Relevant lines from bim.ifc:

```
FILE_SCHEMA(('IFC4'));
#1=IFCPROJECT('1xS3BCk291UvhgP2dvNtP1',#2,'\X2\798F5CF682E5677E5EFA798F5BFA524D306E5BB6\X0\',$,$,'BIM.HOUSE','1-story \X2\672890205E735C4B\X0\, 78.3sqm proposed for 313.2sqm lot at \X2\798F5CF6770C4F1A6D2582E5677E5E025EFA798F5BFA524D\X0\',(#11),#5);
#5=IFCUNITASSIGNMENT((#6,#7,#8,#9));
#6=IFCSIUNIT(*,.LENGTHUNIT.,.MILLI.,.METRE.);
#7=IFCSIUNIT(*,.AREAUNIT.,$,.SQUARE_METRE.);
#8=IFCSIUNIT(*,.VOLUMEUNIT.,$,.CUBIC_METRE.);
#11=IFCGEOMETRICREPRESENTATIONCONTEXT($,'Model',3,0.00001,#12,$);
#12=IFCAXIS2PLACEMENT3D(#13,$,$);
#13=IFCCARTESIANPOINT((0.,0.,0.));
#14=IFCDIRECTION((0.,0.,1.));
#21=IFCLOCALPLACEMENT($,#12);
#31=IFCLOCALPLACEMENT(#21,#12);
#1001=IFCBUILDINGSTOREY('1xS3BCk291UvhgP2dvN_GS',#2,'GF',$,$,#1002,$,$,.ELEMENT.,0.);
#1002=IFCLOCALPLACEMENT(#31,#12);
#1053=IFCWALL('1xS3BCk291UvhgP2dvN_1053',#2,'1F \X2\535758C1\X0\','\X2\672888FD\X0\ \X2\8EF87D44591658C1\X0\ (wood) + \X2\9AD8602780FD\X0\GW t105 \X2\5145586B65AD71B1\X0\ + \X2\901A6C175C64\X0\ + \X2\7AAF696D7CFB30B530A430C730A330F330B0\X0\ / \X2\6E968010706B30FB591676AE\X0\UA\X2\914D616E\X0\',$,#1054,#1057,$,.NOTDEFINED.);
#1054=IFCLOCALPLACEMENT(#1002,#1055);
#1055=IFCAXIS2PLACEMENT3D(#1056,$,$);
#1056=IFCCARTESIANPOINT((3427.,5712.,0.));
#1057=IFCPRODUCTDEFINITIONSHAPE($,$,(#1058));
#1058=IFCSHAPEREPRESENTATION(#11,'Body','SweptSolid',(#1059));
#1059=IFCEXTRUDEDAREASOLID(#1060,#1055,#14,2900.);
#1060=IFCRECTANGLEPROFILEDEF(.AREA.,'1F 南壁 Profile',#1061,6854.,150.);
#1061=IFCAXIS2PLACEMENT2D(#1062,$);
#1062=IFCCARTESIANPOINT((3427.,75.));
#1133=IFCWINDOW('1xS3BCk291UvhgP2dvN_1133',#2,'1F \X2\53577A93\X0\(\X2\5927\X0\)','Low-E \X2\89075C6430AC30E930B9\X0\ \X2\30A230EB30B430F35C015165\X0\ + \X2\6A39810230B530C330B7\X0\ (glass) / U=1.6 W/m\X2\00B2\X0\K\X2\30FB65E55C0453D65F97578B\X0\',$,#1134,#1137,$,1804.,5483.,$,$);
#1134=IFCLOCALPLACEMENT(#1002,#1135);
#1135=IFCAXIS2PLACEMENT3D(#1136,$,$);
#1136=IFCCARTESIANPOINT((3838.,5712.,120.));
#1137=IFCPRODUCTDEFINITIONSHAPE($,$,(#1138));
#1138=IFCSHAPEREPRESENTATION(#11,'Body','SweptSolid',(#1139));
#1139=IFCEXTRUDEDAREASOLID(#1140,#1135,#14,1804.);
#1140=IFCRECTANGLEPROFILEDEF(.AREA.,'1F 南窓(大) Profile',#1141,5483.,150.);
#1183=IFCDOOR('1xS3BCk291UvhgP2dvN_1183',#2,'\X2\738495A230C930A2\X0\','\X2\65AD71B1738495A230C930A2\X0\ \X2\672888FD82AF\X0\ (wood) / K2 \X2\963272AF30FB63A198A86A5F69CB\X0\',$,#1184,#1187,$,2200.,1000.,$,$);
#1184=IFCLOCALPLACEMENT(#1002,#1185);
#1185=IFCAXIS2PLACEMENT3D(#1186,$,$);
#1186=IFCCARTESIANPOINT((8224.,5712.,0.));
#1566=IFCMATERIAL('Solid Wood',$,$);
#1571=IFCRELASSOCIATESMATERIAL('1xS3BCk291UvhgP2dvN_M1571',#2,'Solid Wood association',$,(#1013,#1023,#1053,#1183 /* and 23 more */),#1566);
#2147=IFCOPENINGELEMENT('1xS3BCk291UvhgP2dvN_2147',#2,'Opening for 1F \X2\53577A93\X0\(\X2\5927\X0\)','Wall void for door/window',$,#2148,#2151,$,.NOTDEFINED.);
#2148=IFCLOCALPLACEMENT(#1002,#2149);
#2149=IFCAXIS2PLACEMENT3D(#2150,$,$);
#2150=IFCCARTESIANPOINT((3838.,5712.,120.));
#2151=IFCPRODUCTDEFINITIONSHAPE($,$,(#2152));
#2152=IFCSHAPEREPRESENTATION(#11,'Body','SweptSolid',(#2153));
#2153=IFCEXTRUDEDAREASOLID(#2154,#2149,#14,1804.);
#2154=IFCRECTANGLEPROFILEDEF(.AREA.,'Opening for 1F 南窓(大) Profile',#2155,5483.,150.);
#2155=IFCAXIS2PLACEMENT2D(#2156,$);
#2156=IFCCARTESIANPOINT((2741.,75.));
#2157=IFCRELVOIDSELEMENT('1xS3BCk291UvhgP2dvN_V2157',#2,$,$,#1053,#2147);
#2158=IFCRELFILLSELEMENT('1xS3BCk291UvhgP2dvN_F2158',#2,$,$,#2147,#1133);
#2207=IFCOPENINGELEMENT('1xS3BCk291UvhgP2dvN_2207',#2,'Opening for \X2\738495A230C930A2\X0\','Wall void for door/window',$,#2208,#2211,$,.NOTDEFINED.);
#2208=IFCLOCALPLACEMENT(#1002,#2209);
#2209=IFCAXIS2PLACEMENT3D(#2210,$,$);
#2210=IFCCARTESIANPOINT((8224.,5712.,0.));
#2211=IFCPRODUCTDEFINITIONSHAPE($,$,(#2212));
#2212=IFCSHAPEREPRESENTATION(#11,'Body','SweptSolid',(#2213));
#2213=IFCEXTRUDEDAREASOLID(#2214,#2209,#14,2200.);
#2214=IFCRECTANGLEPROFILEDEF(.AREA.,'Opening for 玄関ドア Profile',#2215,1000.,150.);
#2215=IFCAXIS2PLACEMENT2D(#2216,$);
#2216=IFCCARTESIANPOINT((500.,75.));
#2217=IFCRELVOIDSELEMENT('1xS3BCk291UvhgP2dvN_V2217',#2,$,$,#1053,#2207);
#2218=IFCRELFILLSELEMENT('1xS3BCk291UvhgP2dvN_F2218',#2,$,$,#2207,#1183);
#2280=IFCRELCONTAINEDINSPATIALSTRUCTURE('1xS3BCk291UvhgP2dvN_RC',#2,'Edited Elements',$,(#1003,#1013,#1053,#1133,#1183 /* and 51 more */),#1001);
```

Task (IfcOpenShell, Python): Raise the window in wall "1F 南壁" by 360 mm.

```python
import numpy as np
import ifcopenshell
import ifcopenshell.api.geometry
import ifcopenshell.util.placement
import ifcopenshell.util.unit

model = ifcopenshell.open("bim.ifc")
unit_scale = ifcopenshell.util.unit.calculate_unit_scale(model)

window = model.by_guid("1xS3BCk291UvhgP2dvN_1133")
opening = window.FillsVoids[0].RelatingOpeningElement
dz = 0.36 / unit_scale

shift = np.array([0.0, 0.0, dz])
# The window is not placed relative to its opening, so move both.
for product in (opening, window):
    matrix = ifcopenshell.util.placement.get_local_placement(product.ObjectPlacement)
    matrix[:3, 3] += shift
    ifcopenshell.api.geometry.edit_object_placement(model, product=product, matrix=matrix, is_si=False)

print(f"moved by {dz * unit_scale:+.3f} m")

model.write("bim_rev.ifc")
```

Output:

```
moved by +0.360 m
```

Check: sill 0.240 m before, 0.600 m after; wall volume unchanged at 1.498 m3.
